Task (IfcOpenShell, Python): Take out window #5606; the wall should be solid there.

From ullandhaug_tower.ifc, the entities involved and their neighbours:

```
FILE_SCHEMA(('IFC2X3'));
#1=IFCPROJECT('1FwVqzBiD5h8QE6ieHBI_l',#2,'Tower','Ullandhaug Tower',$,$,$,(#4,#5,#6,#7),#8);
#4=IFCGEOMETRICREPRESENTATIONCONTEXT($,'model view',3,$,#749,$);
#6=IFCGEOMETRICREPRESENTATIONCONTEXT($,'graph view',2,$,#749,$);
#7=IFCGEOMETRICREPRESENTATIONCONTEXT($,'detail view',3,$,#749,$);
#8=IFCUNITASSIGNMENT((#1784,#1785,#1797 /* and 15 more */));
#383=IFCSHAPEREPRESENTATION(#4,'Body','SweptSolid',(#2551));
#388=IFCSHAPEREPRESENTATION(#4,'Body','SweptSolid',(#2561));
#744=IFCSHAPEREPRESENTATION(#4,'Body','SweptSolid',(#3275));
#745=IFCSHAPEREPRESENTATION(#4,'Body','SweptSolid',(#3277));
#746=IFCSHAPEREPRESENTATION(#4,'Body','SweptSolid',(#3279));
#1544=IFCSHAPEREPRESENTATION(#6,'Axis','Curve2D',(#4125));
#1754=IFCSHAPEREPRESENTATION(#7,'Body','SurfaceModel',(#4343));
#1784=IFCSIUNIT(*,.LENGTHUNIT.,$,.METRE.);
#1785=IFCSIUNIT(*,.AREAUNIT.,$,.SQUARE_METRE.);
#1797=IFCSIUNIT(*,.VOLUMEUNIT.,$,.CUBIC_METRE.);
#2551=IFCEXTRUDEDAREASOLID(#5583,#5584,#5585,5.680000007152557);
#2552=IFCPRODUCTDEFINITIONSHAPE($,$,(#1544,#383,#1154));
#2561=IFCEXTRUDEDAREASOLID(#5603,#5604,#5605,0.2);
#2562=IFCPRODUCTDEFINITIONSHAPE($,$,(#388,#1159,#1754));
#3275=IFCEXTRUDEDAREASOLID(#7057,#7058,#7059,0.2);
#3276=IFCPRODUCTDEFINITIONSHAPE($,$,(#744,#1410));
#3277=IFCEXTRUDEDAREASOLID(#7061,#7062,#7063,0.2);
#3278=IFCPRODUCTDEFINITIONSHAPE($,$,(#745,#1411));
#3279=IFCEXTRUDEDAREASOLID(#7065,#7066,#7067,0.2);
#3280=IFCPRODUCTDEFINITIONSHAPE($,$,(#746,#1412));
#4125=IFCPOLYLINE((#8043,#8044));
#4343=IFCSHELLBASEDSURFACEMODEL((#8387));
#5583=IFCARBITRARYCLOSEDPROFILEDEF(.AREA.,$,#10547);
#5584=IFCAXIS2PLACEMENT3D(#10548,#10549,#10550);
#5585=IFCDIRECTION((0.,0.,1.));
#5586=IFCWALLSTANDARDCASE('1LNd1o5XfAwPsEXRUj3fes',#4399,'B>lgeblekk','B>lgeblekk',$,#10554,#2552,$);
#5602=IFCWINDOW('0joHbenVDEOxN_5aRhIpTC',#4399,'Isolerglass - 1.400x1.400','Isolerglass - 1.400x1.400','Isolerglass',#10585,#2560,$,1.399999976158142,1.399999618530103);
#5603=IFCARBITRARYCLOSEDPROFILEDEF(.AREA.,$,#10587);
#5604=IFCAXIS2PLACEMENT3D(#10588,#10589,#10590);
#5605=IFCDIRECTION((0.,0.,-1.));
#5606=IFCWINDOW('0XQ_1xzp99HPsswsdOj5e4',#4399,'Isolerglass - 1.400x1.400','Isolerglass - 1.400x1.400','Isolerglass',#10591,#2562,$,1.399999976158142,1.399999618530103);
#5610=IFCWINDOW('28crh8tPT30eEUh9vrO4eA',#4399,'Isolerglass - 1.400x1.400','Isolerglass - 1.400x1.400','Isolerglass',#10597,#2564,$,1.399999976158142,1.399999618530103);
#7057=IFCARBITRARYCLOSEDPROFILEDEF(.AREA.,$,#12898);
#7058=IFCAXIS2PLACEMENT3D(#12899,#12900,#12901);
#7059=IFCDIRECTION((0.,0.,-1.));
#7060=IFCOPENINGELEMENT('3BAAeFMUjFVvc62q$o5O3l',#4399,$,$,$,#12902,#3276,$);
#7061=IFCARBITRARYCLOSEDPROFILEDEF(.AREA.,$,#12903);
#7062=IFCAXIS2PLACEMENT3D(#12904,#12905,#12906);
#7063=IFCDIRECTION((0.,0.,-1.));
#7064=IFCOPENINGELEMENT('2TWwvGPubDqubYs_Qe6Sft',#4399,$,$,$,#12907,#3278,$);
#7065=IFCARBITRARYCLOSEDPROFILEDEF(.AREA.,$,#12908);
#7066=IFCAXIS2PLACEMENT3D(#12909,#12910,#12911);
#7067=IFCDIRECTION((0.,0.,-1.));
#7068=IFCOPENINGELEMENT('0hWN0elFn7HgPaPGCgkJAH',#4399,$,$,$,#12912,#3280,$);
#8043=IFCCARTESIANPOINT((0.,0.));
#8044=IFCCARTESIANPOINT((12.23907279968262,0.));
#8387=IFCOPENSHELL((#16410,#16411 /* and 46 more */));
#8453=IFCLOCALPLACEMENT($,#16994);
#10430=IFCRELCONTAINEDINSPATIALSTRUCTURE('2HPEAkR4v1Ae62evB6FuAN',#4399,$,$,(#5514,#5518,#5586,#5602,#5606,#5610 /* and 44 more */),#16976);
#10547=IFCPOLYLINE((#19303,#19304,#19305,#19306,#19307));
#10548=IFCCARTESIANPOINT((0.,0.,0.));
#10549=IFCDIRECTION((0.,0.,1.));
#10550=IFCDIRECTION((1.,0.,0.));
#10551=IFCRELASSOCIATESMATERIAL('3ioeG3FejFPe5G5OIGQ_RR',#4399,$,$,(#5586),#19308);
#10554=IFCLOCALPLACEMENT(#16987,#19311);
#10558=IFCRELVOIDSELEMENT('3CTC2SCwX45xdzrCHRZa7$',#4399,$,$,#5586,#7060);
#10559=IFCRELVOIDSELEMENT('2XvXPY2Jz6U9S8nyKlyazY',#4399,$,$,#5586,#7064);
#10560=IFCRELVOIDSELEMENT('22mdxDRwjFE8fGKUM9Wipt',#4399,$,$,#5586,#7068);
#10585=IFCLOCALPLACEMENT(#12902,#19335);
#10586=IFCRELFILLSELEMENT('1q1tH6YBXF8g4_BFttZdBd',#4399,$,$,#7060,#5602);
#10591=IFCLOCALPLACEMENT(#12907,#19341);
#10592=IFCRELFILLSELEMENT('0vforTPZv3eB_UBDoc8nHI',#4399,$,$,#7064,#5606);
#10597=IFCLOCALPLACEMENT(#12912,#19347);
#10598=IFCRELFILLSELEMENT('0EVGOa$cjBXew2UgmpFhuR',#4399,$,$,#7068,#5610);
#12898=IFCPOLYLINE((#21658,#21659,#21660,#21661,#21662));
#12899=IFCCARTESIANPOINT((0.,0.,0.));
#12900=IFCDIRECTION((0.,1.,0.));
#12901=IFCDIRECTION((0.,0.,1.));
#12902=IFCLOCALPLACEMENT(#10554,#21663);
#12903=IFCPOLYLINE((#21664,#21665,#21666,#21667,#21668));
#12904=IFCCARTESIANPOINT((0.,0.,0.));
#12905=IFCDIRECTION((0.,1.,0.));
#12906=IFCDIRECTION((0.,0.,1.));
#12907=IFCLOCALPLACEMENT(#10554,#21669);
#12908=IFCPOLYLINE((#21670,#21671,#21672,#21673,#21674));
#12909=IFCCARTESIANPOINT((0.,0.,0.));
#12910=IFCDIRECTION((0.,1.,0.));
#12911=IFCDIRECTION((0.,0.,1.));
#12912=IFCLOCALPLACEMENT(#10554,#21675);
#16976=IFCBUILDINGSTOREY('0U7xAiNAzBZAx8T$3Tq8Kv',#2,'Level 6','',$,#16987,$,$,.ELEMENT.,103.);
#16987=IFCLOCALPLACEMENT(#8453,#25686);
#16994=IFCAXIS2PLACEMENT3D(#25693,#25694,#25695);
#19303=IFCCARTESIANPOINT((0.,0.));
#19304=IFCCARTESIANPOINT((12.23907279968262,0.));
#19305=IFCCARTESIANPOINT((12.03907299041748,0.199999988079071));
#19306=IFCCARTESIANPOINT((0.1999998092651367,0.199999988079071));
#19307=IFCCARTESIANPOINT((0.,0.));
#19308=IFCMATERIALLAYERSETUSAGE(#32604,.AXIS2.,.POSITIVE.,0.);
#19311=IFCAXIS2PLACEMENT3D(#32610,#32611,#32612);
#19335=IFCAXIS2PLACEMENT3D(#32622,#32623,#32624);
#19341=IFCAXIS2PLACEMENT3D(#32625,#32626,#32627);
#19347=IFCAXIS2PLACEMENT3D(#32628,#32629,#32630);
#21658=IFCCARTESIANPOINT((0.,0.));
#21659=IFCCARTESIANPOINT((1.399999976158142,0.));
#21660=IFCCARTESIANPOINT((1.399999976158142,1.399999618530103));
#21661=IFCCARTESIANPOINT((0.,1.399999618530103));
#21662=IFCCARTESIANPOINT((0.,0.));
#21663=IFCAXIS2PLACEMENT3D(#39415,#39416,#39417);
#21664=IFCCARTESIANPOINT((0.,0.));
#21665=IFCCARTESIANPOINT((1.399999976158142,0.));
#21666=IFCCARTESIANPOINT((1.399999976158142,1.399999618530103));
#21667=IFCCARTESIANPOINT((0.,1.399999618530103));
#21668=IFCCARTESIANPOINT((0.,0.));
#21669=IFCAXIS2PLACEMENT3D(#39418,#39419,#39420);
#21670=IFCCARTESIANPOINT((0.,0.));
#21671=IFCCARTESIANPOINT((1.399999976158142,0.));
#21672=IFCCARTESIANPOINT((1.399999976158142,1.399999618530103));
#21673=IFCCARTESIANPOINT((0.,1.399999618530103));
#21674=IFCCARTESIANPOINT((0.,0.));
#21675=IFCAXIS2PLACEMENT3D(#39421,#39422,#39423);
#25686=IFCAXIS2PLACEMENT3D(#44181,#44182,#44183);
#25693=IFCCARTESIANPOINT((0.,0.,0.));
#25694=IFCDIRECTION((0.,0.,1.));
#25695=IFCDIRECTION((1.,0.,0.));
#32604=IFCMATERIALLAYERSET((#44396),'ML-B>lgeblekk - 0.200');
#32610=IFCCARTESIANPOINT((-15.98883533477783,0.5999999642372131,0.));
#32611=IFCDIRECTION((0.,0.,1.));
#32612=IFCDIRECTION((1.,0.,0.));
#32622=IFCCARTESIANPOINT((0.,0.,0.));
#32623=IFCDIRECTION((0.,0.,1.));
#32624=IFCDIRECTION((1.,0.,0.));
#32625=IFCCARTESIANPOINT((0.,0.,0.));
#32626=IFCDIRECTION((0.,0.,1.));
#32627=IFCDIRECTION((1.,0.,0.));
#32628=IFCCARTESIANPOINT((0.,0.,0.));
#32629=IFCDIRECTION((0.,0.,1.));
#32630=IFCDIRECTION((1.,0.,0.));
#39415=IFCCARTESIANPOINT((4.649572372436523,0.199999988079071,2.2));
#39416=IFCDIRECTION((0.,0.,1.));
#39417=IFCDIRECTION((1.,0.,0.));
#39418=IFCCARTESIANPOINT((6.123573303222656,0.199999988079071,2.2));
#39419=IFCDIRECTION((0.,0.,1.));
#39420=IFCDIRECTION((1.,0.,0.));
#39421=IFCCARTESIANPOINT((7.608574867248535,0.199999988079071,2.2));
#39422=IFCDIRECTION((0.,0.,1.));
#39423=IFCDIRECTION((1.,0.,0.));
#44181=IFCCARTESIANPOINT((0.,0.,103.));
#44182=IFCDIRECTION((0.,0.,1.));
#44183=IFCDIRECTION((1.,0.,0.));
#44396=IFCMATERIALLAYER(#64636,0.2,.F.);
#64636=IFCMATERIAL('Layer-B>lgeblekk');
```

```python
import ifcopenshell
import ifcopenshell.api.feature
import ifcopenshell.api.root
import ifcopenshell.geom
import ifcopenshell.util.shape

model = ifcopenshell.open("ullandhaug_tower.ifc")
settings = ifcopenshell.geom.settings()


def volume(element):
    """Net volume in cubic metres, openings subtracted."""
    shape = ifcopenshell.geom.create_shape(settings, element)
    return ifcopenshell.util.shape.get_volume(shape.geometry)


window = model.by_guid("0XQ_1xzp99HPsswsdOj5e4")
opening = window.FillsVoids[0].RelatingOpeningElement
wall = opening.VoidsElements[0].RelatingBuildingElement
before = volume(wall)

ifcopenshell.api.root.remove_product(model, product=window)
ifcopenshell.api.feature.remove_feature(model, feature=opening)

after = volume(wall)

print(f"wall volume {before:.3f} -> {after:.3f} m3")

model.write("ullandhaug_tower_updated.ifc")
```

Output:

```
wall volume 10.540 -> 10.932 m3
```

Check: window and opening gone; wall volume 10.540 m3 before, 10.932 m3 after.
